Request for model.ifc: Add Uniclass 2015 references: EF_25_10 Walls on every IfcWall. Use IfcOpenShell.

First a look at what the model holds.

```python
import ifcopenshell

model = ifcopenshell.open("model.ifc")
print(model.schema)
print("classifications:", [c.Name for c in model.by_type("IfcClassification")])
for ifc_class in ("IfcDoor", "IfcRoof", "IfcStair", "IfcWall", "IfcWindow"):
    print(ifc_class, len(model.by_type(ifc_class)))
```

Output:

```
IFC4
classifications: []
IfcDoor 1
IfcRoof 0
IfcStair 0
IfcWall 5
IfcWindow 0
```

```python
import ifcopenshell
import ifcopenshell.api.classification

model = ifcopenshell.open("model.ifc")

system = ifcopenshell.api.classification.add_classification(model, classification="Uniclass 2015")

codes = {
    "IfcWall": ("EF_25_10", "Walls"),
}
for ifc_class, (code, name) in codes.items():
    products = model.by_type(ifc_class)
    ifcopenshell.api.classification.add_reference(
        model, products=products, classification=system, identification=code, name=name
    )
    print(code, len(products))

model.write("model_edited.ifc")
```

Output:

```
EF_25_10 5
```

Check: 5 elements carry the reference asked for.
